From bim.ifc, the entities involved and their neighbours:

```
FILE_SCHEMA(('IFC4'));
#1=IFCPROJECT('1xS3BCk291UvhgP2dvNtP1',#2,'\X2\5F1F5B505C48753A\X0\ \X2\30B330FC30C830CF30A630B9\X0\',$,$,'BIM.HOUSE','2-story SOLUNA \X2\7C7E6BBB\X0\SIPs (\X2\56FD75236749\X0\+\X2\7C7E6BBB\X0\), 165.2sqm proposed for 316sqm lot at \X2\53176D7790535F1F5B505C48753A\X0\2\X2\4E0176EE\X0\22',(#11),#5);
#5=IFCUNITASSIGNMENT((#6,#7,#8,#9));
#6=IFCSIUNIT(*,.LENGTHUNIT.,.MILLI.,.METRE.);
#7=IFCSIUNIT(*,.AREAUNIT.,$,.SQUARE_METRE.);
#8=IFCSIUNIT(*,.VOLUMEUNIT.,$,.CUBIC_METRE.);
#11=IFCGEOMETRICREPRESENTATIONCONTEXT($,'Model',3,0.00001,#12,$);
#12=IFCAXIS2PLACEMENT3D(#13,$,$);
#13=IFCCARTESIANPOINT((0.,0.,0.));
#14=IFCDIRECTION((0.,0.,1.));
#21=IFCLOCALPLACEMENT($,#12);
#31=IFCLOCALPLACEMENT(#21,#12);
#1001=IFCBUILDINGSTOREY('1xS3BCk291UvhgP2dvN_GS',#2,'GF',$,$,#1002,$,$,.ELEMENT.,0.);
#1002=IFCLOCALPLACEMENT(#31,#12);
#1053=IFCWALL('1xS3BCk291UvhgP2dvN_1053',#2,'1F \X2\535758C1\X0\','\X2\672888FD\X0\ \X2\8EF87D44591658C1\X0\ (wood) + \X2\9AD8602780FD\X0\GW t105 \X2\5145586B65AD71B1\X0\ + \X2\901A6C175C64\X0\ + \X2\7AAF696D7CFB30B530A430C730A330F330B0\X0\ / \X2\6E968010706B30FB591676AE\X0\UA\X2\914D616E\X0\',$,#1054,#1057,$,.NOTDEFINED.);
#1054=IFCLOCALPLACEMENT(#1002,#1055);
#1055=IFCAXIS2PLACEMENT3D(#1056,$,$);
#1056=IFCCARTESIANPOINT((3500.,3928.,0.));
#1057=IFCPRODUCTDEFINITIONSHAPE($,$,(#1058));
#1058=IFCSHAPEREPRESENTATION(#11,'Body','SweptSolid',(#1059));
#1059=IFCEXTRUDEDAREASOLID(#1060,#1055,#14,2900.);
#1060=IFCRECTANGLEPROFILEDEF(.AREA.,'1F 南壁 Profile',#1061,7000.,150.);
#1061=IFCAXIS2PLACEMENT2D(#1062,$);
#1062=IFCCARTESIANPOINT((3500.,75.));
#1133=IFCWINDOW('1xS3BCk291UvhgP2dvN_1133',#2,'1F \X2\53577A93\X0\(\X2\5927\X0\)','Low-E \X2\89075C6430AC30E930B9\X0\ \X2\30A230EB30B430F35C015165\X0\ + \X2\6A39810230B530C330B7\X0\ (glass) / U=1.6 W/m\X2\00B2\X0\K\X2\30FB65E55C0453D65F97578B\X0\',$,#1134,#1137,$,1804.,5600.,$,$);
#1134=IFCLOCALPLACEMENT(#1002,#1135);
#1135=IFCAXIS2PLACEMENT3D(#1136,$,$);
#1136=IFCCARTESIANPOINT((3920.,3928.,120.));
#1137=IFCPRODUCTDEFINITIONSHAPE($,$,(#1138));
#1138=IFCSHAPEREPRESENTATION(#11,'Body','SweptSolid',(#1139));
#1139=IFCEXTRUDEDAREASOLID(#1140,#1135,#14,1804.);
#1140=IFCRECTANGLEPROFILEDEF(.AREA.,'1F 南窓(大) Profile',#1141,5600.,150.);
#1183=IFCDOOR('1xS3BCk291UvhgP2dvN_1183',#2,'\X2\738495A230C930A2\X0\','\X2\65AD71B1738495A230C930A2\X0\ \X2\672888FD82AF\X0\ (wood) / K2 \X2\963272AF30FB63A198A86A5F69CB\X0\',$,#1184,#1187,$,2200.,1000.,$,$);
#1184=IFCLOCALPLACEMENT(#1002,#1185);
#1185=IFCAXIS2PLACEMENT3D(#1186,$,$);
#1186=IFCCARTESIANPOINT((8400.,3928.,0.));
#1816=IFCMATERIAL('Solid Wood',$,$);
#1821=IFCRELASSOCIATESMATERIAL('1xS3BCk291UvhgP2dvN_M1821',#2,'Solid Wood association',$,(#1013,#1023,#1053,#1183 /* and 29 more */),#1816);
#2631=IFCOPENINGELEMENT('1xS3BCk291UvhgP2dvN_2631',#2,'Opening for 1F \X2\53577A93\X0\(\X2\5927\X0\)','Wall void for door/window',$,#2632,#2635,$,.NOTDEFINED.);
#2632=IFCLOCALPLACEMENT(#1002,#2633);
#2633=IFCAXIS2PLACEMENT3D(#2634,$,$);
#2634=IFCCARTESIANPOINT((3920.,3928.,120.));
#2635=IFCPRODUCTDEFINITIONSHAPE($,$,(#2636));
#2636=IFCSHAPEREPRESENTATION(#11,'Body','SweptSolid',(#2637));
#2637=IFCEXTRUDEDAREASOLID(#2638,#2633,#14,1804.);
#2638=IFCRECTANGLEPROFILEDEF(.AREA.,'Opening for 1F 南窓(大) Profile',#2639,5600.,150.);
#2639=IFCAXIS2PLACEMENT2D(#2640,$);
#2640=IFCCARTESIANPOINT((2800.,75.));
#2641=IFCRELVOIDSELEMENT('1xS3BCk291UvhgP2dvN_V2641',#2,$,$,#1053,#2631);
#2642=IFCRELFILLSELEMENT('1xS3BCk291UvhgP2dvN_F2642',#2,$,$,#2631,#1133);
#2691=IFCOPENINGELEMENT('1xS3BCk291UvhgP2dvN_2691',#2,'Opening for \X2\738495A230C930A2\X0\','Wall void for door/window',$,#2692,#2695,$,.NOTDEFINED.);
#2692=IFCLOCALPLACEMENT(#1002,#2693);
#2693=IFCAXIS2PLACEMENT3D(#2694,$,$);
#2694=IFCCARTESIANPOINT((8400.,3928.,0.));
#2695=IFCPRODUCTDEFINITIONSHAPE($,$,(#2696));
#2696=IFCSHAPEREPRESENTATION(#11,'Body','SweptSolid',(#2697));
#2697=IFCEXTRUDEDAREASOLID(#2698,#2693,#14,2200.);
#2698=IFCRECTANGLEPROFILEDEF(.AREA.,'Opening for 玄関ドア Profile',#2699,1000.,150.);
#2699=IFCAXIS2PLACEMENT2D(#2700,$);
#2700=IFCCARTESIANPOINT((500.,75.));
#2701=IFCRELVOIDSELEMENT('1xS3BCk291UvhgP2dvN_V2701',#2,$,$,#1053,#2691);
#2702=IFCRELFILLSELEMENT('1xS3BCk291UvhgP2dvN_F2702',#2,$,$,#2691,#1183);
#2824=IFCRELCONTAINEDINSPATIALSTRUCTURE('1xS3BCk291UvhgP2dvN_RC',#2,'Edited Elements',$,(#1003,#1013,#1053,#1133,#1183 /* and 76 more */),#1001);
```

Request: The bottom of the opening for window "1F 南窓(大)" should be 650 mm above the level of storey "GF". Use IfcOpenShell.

```python
import numpy as np
import ifcopenshell
import ifcopenshell.api.geometry
import ifcopenshell.geom
import ifcopenshell.util.element
import ifcopenshell.util.placement
import ifcopenshell.util.shape
import ifcopenshell.util.unit

model = ifcopenshell.open("bim.ifc")
unit_scale = ifcopenshell.util.unit.calculate_unit_scale(model)

window = model.by_guid("1xS3BCk291UvhgP2dvN_1133")
opening = window.FillsVoids[0].RelatingOpeningElement
storey = ifcopenshell.util.element.get_container(window, ifc_class="IfcBuildingStorey")
level = ifcopenshell.util.placement.get_local_placement(storey.ObjectPlacement)[2, 3]

# The opening's origin need not be at the sill, so measure its lowest point.
shape = ifcopenshell.geom.create_shape(ifcopenshell.geom.settings(), opening)
bottom = ifcopenshell.util.shape.get_shape_bottom_elevation(shape, shape.geometry) / unit_scale
dz = level + 0.65 / unit_scale - bottom

shift = np.array([0.0, 0.0, dz])
# The window is not placed relative to its opening, so move both.
for product in (opening, window):
    matrix = ifcopenshell.util.placement.get_local_placement(product.ObjectPlacement)
    matrix[:3, 3] += shift
    ifcopenshell.api.geometry.edit_object_placement(model, product=product, matrix=matrix, is_si=False)

print(f"moved by {dz * unit_scale:+.3f} m")

model.write("bim_rev.ifc")
```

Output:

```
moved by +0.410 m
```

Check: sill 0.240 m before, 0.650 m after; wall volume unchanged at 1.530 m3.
